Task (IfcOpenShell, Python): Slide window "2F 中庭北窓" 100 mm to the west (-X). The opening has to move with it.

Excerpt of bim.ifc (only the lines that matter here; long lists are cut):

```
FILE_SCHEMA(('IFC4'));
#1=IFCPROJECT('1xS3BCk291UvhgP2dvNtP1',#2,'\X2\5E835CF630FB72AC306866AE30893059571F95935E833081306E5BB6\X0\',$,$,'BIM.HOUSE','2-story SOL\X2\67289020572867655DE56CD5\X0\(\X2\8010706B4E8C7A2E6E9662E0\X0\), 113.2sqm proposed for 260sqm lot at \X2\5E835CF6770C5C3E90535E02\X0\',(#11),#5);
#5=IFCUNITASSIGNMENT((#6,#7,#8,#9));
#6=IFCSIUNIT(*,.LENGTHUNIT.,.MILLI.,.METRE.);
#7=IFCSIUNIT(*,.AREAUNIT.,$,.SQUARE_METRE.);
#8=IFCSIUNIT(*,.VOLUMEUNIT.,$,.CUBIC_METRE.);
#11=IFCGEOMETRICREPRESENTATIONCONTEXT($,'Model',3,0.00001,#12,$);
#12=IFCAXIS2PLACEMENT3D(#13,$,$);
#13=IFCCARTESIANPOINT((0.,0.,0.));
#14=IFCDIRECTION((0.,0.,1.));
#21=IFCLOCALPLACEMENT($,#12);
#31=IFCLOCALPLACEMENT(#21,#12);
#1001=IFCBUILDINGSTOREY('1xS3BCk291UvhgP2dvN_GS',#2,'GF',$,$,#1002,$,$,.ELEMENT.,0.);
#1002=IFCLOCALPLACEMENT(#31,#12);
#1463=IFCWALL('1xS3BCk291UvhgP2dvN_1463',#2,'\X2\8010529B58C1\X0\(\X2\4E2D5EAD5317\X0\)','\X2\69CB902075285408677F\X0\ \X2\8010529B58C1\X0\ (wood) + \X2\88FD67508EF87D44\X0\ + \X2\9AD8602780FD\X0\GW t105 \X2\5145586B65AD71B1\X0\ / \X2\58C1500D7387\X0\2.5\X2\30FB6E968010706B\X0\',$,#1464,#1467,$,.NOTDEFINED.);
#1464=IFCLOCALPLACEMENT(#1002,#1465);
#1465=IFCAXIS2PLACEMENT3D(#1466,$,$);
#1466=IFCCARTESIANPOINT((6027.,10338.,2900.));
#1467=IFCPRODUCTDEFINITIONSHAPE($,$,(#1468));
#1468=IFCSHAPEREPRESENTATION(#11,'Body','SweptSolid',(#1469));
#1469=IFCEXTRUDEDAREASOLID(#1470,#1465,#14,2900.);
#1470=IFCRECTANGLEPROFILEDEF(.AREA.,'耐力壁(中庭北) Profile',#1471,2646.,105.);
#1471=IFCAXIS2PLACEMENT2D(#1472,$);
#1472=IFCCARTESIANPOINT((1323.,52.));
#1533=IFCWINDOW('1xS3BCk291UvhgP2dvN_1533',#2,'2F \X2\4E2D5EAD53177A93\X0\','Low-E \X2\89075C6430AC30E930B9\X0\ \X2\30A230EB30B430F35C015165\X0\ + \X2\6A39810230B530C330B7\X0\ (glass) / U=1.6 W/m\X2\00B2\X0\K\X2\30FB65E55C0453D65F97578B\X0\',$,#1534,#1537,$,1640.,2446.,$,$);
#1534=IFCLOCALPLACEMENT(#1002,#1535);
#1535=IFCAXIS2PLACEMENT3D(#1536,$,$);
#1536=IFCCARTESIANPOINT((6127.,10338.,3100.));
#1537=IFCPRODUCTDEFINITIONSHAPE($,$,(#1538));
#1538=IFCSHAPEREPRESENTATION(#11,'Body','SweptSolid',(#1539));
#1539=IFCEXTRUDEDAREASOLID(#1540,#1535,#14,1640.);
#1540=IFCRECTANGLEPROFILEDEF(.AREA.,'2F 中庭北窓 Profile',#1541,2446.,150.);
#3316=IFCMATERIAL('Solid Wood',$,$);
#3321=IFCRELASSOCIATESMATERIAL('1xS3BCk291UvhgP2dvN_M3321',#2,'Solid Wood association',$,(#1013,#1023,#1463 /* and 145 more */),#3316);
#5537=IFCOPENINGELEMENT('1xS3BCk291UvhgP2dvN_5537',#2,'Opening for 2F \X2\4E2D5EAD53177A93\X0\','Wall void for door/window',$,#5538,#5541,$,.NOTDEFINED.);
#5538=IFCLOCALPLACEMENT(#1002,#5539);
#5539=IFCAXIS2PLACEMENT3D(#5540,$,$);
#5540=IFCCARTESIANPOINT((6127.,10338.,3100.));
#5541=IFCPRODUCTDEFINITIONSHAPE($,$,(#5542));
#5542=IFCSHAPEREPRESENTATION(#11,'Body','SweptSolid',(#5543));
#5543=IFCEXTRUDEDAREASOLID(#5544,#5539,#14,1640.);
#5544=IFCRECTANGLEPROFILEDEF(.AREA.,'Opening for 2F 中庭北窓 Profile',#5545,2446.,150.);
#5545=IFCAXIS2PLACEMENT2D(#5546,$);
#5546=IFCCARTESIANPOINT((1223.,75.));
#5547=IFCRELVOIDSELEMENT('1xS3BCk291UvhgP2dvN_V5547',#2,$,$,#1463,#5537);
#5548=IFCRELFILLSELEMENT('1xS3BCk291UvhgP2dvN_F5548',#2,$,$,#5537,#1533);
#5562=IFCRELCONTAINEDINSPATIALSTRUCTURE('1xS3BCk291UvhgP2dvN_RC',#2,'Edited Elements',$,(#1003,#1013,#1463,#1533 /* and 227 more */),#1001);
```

```python
import ifcopenshell
import ifcopenshell.api.geometry
import ifcopenshell.util.placement

model = ifcopenshell.open("bim.ifc")

window = model.by_id(1533)
opening = window.FillsVoids[0].RelatingOpeningElement
wall = opening.VoidsElements[0].RelatingBuildingElement

wall_matrix = ifcopenshell.util.placement.get_local_placement(wall.ObjectPlacement)
shift = wall_matrix[:3, 0] * -100.0
before = ifcopenshell.util.placement.get_local_placement(window.ObjectPlacement)[:3, 3].copy()

# The window is not placed relative to its opening, so move both.
for product in (opening, window):
    matrix = ifcopenshell.util.placement.get_local_placement(product.ObjectPlacement)
    matrix[:3, 3] += shift
    ifcopenshell.api.geometry.edit_object_placement(model, product=product, matrix=matrix, is_si=False)

after = ifcopenshell.util.placement.get_local_placement(window.ObjectPlacement)[:3, 3]
print("window moved by", (after - before).round(3) + 0.0)

model.write("bim_edited.ifc")
```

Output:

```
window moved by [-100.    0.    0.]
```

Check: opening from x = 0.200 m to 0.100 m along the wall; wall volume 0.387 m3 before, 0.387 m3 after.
